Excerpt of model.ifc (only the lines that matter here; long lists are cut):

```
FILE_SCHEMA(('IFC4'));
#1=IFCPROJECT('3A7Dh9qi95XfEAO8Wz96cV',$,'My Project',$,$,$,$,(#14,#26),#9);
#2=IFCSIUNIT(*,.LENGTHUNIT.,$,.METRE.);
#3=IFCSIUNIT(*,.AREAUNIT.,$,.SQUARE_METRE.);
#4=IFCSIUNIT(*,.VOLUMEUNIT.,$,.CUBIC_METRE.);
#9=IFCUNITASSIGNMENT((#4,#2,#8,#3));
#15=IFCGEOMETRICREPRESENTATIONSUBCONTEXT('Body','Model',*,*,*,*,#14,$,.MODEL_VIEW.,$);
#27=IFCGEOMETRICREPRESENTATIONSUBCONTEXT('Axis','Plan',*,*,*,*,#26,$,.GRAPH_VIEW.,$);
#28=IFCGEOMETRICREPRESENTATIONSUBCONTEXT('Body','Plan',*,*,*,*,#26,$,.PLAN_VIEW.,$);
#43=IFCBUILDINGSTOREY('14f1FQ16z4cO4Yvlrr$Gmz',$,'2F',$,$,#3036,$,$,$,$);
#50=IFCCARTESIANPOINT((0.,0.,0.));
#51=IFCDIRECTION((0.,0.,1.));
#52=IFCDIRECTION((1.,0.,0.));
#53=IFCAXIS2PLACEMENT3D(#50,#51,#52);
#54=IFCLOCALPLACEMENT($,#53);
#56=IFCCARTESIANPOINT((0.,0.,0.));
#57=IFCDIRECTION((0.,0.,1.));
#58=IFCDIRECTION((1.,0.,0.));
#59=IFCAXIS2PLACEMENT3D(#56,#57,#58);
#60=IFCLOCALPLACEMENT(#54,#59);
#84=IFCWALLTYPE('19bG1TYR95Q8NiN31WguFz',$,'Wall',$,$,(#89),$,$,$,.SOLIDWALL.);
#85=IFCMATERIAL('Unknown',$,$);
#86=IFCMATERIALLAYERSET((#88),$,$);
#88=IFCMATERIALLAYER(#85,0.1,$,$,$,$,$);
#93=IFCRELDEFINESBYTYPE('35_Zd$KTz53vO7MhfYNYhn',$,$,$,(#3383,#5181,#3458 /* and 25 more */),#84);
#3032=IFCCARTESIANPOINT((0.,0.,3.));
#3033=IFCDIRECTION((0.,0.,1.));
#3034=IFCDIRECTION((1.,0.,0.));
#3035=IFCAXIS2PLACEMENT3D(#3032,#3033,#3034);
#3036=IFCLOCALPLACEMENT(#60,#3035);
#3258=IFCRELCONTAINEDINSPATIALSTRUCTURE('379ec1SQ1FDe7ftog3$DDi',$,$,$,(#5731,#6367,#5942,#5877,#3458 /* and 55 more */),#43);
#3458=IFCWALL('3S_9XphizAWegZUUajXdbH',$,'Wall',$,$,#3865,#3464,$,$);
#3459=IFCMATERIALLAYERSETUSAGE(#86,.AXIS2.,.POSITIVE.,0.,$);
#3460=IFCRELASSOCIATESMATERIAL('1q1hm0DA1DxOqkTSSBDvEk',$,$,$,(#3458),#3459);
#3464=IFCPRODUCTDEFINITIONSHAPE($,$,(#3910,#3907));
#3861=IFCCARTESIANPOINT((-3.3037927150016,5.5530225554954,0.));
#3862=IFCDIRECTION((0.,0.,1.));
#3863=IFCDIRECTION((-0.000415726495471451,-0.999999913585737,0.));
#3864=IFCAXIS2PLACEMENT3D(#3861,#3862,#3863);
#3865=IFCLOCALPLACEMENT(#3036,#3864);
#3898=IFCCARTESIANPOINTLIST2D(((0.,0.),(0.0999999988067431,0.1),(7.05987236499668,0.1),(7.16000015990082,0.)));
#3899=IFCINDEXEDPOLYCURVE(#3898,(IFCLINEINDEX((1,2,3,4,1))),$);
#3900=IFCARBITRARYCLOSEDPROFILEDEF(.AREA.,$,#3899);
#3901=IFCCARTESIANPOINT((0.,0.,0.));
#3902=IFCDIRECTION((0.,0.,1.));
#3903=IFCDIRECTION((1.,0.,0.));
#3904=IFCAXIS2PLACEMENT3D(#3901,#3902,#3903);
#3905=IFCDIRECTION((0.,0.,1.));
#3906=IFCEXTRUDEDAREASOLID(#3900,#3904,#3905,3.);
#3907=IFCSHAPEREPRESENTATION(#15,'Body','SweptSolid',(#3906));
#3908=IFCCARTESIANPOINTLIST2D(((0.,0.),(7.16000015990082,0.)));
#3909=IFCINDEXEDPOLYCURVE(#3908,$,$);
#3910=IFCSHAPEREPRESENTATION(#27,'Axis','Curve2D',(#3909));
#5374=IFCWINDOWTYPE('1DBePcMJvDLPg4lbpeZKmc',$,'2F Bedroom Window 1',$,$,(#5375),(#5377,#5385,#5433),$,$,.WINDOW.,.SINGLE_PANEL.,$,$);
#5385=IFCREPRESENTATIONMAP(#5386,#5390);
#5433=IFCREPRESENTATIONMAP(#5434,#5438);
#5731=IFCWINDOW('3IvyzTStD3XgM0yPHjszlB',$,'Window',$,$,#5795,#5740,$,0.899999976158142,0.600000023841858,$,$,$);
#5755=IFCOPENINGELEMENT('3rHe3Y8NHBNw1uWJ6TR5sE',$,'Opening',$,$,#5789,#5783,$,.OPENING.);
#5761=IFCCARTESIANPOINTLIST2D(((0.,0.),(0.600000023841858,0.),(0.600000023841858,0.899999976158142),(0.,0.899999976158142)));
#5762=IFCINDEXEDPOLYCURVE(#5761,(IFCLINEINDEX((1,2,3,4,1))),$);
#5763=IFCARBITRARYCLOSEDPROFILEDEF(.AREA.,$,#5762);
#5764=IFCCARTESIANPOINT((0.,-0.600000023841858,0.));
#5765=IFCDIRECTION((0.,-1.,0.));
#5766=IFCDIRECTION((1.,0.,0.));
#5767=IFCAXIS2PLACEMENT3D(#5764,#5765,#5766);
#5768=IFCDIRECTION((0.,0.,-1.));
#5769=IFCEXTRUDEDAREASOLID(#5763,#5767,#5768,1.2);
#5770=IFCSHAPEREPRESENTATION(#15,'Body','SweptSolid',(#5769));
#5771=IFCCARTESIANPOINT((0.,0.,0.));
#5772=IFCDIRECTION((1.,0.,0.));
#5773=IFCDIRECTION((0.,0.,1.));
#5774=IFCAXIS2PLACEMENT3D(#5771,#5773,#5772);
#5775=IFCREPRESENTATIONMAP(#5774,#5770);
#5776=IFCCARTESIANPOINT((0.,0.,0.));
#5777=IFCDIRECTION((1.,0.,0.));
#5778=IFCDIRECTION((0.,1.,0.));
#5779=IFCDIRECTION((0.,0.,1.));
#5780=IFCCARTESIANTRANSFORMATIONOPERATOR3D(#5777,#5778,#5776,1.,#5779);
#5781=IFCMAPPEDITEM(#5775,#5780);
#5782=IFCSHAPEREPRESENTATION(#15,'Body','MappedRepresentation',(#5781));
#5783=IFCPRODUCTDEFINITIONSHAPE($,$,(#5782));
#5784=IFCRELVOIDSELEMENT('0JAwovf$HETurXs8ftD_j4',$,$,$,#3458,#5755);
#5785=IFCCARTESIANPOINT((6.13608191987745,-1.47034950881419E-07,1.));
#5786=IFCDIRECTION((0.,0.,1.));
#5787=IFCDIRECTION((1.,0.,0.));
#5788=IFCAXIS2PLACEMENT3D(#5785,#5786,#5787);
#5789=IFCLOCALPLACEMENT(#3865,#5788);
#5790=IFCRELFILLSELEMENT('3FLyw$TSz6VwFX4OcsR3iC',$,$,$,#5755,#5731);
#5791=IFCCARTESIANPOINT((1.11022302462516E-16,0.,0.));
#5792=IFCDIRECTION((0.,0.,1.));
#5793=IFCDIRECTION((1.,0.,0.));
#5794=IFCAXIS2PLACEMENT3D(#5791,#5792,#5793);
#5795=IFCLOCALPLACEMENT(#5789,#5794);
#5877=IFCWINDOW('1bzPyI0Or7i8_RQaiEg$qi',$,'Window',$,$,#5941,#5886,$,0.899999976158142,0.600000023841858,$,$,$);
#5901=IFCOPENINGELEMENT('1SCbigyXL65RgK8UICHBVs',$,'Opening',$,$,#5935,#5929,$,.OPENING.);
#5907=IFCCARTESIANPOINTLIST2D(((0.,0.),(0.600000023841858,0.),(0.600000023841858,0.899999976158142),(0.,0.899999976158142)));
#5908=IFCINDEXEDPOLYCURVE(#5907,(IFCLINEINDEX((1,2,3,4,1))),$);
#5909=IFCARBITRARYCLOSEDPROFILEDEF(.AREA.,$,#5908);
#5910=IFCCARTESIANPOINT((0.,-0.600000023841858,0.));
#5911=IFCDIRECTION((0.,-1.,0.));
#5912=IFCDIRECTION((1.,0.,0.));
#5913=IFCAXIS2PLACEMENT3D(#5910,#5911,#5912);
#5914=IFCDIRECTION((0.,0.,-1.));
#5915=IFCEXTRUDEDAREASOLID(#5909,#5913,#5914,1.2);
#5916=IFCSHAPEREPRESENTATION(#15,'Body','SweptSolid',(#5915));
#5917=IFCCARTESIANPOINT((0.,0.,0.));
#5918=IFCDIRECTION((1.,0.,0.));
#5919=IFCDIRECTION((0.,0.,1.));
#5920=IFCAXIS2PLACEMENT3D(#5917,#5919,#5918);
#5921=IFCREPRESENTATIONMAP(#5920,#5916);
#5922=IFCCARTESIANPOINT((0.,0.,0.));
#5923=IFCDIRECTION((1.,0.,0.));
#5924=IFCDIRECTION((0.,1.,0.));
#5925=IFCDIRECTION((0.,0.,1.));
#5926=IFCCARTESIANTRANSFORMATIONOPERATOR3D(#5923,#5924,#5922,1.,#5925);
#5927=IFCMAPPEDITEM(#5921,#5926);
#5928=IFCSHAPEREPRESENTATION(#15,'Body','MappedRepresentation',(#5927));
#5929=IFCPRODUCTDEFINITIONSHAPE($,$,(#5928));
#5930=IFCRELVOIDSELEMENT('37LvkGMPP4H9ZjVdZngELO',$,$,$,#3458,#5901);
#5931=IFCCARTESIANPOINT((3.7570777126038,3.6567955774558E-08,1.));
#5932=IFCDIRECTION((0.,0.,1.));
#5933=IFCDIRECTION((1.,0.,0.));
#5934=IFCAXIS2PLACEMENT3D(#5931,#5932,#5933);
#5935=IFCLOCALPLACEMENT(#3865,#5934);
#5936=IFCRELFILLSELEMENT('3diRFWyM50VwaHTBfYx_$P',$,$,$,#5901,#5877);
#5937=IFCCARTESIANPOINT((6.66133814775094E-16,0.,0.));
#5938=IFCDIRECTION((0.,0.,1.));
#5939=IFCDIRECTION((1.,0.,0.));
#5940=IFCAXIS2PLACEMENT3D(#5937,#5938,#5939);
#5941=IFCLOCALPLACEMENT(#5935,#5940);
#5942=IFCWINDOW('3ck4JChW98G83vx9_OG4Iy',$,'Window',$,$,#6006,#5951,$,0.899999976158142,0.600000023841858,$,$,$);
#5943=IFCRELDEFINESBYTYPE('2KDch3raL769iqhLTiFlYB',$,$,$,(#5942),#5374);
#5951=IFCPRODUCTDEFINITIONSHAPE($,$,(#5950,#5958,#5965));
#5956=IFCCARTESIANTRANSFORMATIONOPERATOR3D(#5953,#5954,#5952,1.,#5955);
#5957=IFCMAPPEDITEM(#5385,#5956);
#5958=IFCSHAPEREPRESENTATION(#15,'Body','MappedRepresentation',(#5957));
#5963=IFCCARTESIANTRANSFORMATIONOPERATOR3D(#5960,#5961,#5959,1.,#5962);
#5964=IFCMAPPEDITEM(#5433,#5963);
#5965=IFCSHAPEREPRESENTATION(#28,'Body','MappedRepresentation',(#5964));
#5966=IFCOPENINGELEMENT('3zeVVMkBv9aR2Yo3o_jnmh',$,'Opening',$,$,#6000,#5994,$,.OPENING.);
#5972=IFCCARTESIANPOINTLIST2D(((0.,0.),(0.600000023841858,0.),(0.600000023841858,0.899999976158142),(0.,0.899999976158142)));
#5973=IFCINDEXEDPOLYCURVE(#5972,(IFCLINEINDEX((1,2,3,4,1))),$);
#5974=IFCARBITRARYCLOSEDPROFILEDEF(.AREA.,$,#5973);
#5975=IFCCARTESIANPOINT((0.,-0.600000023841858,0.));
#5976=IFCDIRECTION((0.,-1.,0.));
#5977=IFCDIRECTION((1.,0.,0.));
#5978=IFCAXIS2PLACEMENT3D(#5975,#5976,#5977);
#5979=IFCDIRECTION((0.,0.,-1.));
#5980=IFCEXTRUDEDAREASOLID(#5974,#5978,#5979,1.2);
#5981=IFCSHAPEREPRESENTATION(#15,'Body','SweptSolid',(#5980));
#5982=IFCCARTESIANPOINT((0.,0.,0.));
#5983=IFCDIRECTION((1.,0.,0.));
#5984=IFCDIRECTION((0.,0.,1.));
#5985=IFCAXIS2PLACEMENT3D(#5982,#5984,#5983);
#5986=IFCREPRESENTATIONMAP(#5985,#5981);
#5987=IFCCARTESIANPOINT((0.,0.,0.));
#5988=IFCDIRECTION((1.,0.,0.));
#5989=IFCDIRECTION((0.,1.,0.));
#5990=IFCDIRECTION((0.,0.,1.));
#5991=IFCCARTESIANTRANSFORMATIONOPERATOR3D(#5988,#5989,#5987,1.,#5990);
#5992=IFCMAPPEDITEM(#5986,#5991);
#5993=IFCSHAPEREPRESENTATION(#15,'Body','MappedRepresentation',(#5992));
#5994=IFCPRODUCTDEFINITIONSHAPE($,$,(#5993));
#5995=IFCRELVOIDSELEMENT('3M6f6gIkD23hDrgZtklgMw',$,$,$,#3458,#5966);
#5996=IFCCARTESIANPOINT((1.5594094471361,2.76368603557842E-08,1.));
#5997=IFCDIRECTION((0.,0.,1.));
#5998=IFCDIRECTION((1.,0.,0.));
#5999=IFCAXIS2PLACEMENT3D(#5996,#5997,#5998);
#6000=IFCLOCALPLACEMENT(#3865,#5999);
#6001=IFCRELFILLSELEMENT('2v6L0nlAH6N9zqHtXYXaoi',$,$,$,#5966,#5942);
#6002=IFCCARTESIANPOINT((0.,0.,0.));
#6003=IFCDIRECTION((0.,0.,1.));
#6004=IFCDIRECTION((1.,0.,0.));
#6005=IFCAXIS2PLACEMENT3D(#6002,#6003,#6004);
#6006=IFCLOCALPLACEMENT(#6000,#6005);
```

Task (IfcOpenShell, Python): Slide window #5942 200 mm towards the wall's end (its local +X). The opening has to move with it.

```python
import ifcopenshell
import ifcopenshell.api.geometry
import ifcopenshell.util.placement

model = ifcopenshell.open("model.ifc")

window = model.by_guid("3ck4JChW98G83vx9_OG4Iy")
opening = window.FillsVoids[0].RelatingOpeningElement
wall = opening.VoidsElements[0].RelatingBuildingElement

wall_matrix = ifcopenshell.util.placement.get_local_placement(wall.ObjectPlacement)
shift = wall_matrix[:3, 0] * 0.2
before = ifcopenshell.util.placement.get_local_placement(window.ObjectPlacement)[:3, 3].copy()

# The window is placed relative to its opening, so it follows when the opening moves.
matrix = ifcopenshell.util.placement.get_local_placement(opening.ObjectPlacement)
matrix[:3, 3] += shift
ifcopenshell.api.geometry.edit_object_placement(
    model, product=opening, matrix=matrix, is_si=False, should_transform_children=True
)

after = ifcopenshell.util.placement.get_local_placement(window.ObjectPlacement)[:3, 3]
print("window moved by", (after - before).round(3) + 0.0)

model.write("model_edited.ifc")
```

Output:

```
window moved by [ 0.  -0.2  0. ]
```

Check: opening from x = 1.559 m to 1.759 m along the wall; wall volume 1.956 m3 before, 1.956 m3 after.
